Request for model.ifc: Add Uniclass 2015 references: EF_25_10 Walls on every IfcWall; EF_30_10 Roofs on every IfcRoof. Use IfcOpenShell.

First a look at what the model holds.

```python
import ifcopenshell

model = ifcopenshell.open("model.ifc")
print(model.schema)
print("classifications:", [c.Name for c in model.by_type("IfcClassification")])
for ifc_class in ("IfcDoor", "IfcRoof", "IfcStair", "IfcWall", "IfcWindow"):
    print(ifc_class, len(model.by_type(ifc_class)))
```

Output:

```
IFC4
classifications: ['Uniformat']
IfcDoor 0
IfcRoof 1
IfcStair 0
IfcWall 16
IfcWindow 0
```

```python
import ifcopenshell
import ifcopenshell.api.classification

model = ifcopenshell.open("model.ifc")

system = ifcopenshell.api.classification.add_classification(model, classification="Uniclass 2015")

codes = {
    "IfcWall": ("EF_25_10", "Walls"),
    "IfcRoof": ("EF_30_10", "Roofs"),
}
for ifc_class, (code, name) in codes.items():
    products = model.by_type(ifc_class)
    ifcopenshell.api.classification.add_reference(
        model, products=products, classification=system, identification=code, name=name
    )
    print(code, len(products))

model.write("model_rev.ifc")
```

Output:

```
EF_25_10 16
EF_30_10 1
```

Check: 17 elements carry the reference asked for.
